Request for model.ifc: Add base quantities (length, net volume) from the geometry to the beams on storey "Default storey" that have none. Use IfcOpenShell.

First a look at what the model holds.

```python
import ifcopenshell
import ifcopenshell.util.element
import ifcopenshell.util.unit

model = ifcopenshell.open("model.ifc")
print(model.schema)
for unit_type in ("LENGTHUNIT", "AREAUNIT", "VOLUMEUNIT"):
    print(unit_type, ifcopenshell.util.unit.calculate_unit_scale(model, unit_type))
storey = next(s for s in model.by_type("IfcBuildingStorey") if s.Name == "Default storey")
beams = [e for e in ifcopenshell.util.element.get_decomposition(storey) if e.is_a("IfcBeam")]
for e in sorted(beams, key=lambda e: e.id()):
    print(e.id(), e.is_a(), e.Name, list(ifcopenshell.util.element.get_psets(e, qtos_only=True)), sep=" | ")
```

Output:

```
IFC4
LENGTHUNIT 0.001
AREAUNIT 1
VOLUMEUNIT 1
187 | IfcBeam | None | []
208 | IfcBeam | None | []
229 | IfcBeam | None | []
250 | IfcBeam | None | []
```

```python
import ifcopenshell
import ifcopenshell.api.pset
import ifcopenshell.geom
import ifcopenshell.util.element
import ifcopenshell.util.shape
import ifcopenshell.util.unit

model = ifcopenshell.open("model.ifc")
unit_scale = ifcopenshell.util.unit.calculate_unit_scale(model)
volume_scale = ifcopenshell.util.unit.calculate_unit_scale(model, "VOLUMEUNIT")
settings = ifcopenshell.geom.settings()

storey = next(s for s in model.by_type("IfcBuildingStorey") if s.Name == "Default storey")
beams = [e for e in ifcopenshell.util.element.get_decomposition(storey) if e.is_a("IfcBeam")]

for e in sorted(beams, key=lambda e: e.id()):
    if ifcopenshell.util.element.get_psets(e, qtos_only=True, should_inherit=False):
        continue
    # Geometry comes back in metres, in the element's own axes.
    shape = ifcopenshell.geom.create_shape(settings, e)
    values = {
        "Length": ifcopenshell.util.shape.get_max_xyz(shape.geometry) / unit_scale,
        "NetVolume": ifcopenshell.util.shape.get_volume(shape.geometry) / volume_scale,
    }
    qto = ifcopenshell.api.pset.add_qto(model, product=e, name="Qto_BeamBaseQuantities")
    ifcopenshell.api.pset.edit_qto(model, qto=qto, properties=values)
    print(e.id(), {k: round(v, 3) for k, v in values.items()})

model.write("model_v2.ifc")
```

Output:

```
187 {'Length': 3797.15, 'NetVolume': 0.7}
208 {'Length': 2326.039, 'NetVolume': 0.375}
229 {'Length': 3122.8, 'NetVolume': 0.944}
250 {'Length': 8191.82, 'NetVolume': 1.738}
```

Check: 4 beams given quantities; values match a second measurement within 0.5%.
